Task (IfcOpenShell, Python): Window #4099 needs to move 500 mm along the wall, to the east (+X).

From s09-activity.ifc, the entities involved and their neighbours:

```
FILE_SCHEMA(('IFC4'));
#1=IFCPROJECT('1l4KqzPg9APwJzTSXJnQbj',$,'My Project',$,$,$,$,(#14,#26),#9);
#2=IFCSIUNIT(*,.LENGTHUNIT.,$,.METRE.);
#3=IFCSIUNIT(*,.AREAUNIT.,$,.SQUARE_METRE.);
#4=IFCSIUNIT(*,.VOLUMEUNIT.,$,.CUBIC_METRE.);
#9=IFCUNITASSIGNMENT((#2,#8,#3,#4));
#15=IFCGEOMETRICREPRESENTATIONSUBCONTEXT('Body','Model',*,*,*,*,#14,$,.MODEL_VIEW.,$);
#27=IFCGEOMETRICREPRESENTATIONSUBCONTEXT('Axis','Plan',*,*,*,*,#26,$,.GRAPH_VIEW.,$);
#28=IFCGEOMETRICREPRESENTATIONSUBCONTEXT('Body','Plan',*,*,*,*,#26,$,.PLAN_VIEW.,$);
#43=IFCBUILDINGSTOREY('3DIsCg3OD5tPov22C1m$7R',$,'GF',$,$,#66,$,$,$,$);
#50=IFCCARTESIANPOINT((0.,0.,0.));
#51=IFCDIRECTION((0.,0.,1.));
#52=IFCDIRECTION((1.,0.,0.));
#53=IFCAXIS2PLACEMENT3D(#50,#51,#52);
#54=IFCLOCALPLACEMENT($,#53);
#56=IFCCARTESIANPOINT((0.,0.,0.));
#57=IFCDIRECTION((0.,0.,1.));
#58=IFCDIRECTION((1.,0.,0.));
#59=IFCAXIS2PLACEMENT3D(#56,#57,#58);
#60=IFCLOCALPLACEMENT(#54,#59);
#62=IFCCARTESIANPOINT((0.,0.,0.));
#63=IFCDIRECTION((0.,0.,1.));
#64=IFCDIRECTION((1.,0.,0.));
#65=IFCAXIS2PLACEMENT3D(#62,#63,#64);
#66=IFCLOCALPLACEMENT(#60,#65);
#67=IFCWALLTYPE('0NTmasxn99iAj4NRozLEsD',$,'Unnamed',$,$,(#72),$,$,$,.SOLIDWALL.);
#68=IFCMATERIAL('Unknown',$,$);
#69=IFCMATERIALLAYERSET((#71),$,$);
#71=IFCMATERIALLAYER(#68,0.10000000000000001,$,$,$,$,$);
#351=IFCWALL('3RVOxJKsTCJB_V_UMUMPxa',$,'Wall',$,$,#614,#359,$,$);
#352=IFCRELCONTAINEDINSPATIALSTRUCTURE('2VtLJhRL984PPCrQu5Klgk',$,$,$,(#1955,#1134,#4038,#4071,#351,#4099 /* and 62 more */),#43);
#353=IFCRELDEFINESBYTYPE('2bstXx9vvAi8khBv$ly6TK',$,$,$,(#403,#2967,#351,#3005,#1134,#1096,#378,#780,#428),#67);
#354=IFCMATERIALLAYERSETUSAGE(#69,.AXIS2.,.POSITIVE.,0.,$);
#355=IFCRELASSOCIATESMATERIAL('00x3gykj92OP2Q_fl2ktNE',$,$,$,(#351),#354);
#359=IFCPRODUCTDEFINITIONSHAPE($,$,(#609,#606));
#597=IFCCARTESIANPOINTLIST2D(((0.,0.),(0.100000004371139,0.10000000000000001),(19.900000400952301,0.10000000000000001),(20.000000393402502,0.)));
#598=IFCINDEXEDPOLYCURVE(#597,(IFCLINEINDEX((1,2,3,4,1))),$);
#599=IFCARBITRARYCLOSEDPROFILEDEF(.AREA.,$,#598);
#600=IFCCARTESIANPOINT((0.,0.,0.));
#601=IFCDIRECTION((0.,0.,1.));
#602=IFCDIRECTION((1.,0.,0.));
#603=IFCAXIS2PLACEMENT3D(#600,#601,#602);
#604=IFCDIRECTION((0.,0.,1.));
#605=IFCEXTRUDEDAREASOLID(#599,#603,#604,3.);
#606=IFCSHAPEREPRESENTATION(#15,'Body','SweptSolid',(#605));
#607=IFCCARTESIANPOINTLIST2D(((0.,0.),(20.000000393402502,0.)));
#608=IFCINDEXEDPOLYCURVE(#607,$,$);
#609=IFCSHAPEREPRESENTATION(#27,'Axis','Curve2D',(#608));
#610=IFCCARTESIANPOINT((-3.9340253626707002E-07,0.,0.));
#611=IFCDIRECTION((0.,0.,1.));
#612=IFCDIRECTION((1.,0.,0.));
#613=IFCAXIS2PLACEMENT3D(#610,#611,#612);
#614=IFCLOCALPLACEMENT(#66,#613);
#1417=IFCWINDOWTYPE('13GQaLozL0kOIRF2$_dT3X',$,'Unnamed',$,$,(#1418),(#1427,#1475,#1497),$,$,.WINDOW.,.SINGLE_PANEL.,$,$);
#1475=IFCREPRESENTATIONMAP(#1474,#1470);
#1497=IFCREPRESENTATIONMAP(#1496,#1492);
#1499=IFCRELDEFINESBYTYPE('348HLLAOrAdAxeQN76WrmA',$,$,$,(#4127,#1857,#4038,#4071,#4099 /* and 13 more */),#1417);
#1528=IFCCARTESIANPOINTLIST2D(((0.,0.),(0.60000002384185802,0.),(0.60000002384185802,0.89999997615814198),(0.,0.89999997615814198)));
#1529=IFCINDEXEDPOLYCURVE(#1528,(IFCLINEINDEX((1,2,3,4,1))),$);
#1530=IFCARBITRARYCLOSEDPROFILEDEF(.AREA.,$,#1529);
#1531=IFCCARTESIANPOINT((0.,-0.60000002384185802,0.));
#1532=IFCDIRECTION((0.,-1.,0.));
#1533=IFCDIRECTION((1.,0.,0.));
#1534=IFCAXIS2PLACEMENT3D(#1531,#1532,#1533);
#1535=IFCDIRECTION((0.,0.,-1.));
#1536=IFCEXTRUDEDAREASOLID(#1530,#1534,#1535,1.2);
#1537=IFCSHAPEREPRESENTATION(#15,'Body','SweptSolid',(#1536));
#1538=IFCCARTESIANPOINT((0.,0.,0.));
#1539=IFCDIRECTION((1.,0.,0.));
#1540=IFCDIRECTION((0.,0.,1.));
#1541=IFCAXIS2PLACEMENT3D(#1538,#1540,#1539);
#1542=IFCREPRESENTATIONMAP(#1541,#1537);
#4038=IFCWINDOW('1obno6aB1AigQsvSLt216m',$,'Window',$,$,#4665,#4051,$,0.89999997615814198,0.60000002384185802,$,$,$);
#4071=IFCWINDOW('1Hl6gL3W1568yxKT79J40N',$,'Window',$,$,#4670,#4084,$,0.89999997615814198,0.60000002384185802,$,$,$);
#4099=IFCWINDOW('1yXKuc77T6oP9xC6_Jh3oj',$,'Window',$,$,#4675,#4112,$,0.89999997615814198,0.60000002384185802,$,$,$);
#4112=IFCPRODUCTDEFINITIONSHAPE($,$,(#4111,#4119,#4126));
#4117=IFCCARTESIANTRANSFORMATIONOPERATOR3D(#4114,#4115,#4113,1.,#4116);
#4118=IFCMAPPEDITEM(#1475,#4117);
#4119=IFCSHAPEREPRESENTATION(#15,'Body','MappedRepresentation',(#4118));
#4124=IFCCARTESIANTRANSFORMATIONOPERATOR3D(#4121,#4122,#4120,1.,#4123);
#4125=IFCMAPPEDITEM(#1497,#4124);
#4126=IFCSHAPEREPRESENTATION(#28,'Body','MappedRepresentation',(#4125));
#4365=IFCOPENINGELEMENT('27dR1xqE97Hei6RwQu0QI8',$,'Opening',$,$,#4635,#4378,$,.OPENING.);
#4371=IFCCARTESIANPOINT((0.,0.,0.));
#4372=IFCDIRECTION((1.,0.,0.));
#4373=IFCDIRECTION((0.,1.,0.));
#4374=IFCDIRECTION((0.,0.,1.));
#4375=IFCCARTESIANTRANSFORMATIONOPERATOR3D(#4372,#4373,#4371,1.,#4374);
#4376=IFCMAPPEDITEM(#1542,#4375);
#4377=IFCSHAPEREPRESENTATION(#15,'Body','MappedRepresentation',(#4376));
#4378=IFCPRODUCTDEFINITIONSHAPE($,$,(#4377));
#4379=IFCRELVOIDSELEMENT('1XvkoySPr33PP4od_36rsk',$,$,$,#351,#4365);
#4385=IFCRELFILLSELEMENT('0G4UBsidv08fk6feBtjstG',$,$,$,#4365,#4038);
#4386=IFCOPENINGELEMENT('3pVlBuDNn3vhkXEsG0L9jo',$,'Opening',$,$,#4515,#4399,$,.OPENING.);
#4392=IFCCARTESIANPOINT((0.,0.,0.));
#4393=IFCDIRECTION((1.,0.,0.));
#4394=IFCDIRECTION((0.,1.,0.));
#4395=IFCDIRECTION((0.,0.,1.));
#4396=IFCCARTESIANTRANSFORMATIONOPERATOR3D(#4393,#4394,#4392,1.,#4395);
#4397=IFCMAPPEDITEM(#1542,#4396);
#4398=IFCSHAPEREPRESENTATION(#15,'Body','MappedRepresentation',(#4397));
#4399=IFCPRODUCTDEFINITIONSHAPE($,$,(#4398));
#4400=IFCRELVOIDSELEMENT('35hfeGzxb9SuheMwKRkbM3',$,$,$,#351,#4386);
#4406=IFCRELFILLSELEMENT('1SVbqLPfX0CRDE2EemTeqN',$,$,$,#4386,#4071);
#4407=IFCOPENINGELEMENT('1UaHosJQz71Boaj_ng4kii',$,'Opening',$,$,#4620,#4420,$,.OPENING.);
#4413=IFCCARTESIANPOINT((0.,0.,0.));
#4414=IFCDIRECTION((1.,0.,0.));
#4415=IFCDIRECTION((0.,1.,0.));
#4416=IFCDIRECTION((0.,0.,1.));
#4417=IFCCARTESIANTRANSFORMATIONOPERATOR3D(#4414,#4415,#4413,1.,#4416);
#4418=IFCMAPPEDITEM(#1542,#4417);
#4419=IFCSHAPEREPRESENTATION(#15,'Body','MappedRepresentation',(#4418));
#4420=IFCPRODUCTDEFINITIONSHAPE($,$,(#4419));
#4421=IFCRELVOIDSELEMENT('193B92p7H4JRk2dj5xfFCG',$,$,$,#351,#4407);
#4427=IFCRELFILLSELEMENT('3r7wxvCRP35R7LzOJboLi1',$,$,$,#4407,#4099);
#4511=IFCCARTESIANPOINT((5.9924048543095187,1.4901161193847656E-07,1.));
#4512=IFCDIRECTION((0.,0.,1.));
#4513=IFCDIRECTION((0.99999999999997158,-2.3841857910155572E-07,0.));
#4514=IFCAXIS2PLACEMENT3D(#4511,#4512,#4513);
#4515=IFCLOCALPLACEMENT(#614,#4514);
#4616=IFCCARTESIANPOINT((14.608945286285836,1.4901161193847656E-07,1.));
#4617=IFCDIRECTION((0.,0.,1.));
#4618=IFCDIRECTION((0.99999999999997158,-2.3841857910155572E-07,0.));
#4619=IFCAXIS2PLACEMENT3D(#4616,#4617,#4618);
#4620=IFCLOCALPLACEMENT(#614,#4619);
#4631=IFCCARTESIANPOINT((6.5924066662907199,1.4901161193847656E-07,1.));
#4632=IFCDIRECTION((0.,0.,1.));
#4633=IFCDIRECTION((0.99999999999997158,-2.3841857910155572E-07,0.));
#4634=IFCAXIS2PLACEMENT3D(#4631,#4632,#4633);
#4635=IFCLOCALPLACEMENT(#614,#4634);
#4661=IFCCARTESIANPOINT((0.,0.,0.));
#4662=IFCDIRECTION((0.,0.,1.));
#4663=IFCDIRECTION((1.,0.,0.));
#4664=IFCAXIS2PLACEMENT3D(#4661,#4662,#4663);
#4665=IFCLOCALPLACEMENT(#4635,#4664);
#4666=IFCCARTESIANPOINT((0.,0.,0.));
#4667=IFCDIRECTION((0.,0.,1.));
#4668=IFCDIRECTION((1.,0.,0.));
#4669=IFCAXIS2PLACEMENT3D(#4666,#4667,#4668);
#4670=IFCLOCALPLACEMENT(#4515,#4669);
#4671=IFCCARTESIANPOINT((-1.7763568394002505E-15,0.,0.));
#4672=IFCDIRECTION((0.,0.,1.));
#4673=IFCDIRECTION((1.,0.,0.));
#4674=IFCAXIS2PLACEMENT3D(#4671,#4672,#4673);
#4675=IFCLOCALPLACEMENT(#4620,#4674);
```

```python
import ifcopenshell
import ifcopenshell.api.geometry
import ifcopenshell.util.placement
import ifcopenshell.util.unit

model = ifcopenshell.open("s09-activity.ifc")
unit_scale = ifcopenshell.util.unit.calculate_unit_scale(model)

window = model.by_id(4099)
opening = window.FillsVoids[0].RelatingOpeningElement
wall = opening.VoidsElements[0].RelatingBuildingElement

wall_matrix = ifcopenshell.util.placement.get_local_placement(wall.ObjectPlacement)
shift = wall_matrix[:3, 0] * 0.5 / unit_scale
before = ifcopenshell.util.placement.get_local_placement(window.ObjectPlacement)[:3, 3].copy()

# The window is placed relative to its opening, so it follows when the opening moves.
matrix = ifcopenshell.util.placement.get_local_placement(opening.ObjectPlacement)
matrix[:3, 3] += shift
ifcopenshell.api.geometry.edit_object_placement(
    model, product=opening, matrix=matrix, is_si=False, should_transform_children=True
)

after = ifcopenshell.util.placement.get_local_placement(window.ObjectPlacement)[:3, 3]
print("window moved by", (after - before).round(3) + 0.0)

model.write("s09-activity_edited.ifc")
```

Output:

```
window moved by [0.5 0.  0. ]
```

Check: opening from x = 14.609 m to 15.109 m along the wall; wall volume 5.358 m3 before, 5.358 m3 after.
